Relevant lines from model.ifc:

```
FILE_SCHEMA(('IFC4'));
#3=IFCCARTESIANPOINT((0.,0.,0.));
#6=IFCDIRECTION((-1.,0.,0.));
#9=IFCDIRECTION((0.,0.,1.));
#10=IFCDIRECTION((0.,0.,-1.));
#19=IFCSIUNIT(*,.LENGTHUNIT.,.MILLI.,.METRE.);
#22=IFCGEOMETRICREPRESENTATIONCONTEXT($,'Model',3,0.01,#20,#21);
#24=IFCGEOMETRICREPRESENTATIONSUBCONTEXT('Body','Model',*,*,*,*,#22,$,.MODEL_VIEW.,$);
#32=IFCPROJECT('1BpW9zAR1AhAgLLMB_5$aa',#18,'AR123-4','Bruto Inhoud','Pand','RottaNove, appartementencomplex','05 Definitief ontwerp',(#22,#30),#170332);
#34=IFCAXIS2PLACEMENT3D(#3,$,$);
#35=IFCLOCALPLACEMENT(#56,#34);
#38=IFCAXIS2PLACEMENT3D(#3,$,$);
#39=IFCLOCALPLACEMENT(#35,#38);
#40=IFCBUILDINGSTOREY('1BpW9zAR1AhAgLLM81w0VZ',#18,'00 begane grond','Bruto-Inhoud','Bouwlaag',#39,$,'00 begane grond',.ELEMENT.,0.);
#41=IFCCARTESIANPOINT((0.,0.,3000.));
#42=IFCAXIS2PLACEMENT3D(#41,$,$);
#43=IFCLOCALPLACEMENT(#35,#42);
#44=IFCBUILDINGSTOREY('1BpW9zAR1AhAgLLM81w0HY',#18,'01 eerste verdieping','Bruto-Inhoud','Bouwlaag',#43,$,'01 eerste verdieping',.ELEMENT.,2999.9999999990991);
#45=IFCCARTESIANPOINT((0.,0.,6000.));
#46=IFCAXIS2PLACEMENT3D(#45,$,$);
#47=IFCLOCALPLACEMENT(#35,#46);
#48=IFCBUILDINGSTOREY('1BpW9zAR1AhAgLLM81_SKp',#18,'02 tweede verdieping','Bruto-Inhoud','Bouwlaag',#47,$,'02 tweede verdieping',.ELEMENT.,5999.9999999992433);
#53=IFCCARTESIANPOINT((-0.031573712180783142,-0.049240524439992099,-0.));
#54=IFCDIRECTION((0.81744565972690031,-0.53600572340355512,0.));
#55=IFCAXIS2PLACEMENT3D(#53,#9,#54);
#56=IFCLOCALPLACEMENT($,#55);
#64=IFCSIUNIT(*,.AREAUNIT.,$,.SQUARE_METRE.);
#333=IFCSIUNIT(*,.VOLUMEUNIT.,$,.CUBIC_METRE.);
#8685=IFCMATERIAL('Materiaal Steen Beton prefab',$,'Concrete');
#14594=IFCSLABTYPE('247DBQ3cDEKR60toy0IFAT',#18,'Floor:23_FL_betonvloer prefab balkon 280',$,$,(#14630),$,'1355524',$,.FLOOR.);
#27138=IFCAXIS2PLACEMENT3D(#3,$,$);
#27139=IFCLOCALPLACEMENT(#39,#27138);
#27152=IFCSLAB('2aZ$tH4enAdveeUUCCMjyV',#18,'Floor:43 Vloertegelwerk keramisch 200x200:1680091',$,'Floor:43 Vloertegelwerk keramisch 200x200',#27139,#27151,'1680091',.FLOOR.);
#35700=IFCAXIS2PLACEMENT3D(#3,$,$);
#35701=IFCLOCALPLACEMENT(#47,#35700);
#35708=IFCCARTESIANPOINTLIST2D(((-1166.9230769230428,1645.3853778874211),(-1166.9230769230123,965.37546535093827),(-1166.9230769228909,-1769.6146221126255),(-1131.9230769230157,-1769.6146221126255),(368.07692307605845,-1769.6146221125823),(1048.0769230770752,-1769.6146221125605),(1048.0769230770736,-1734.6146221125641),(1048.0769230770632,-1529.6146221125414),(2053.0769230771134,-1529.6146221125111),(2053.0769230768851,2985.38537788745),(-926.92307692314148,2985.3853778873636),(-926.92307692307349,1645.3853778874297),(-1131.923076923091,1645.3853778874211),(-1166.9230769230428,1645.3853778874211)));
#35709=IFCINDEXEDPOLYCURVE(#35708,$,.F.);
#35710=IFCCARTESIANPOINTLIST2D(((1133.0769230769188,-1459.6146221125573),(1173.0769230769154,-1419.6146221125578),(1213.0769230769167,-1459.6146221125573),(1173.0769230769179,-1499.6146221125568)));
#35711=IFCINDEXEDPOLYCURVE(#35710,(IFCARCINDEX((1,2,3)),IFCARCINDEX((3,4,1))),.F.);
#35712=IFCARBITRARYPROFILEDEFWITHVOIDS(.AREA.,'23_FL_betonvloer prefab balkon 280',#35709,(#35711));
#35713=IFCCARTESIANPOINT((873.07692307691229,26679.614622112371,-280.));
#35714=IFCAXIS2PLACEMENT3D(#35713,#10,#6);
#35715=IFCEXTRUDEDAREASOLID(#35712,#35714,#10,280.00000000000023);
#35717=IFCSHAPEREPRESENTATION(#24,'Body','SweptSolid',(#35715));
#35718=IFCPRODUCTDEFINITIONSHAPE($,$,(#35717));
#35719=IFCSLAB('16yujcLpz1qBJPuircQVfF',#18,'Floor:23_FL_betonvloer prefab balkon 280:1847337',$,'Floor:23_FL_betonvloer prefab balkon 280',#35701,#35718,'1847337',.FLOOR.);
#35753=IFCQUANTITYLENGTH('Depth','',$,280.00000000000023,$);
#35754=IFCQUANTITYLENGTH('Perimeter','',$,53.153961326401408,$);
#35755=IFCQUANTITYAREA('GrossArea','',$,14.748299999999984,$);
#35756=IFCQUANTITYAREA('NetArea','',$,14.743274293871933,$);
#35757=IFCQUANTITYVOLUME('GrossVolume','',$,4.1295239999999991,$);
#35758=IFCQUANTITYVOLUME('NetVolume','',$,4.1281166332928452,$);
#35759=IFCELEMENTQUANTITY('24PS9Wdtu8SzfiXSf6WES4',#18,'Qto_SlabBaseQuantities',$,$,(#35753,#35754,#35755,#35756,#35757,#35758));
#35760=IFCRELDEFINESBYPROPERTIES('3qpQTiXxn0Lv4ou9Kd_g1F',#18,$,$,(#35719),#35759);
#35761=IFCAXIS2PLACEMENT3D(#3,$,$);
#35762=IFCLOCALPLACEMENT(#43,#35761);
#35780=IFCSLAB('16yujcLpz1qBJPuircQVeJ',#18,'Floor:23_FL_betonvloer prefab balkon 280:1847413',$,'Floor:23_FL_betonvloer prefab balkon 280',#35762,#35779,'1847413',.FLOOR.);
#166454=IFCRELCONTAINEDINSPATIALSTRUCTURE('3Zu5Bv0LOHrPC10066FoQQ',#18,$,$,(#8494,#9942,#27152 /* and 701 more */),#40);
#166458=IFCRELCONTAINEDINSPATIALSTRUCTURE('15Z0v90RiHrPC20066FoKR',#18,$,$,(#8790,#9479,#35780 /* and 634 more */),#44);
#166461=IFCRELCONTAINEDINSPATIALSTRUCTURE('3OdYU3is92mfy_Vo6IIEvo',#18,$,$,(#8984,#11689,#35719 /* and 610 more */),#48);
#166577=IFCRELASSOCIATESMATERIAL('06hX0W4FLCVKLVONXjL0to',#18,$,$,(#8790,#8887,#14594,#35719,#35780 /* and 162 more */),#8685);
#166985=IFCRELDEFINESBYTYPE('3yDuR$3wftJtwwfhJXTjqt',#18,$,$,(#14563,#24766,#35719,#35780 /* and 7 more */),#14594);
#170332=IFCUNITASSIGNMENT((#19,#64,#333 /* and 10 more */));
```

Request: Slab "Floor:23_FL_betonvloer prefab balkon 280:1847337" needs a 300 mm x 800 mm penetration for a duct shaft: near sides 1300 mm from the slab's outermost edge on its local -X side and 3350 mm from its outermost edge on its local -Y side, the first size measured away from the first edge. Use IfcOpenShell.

```python
import numpy as np
import ifcopenshell
import ifcopenshell.api.feature
import ifcopenshell.api.geometry
import ifcopenshell.api.pset
import ifcopenshell.api.root
import ifcopenshell.geom
import ifcopenshell.util.element
import ifcopenshell.util.placement
import ifcopenshell.util.representation
import ifcopenshell.util.shape
import ifcopenshell.util.unit

model = ifcopenshell.open("model.ifc")
unit_scale = ifcopenshell.util.unit.calculate_unit_scale(model)
area_scale = ifcopenshell.util.unit.calculate_unit_scale(model, "AREAUNIT")
volume_scale = ifcopenshell.util.unit.calculate_unit_scale(model, "VOLUMEUNIT")
settings = ifcopenshell.geom.settings()


def volume(element):
    """Net volume in cubic metres, openings subtracted."""
    shape = ifcopenshell.geom.create_shape(settings, element)
    return ifcopenshell.util.shape.get_volume(shape.geometry)


slab = model.by_id(35719)
before = volume(slab)

# Extent in the slab's own axes, in metres. The edges named are its -X and -Y sides.
slab_shape = ifcopenshell.geom.create_shape(settings, slab)
vertices = ifcopenshell.util.shape.get_vertices(slab_shape.geometry)
x_min, y_min, bottom = vertices.min(axis=0)
top = vertices[:, 2].max()

opening = ifcopenshell.api.root.create_entity(model, ifc_class="IfcOpeningElement", name="Duct shaft opening", predefined_type="OPENING")
context = ifcopenshell.util.representation.get_context(model, "Model", "Body", "MODEL_VIEW")
width, depth = 0.3, 0.8
outline = [(0.0, 0.0), (width, 0.0), (width, depth), (0.0, depth), (0.0, 0.0)]
# Overshoot both faces by 50 mm so the cut is clean.
shape = ifcopenshell.api.geometry.add_slab_representation(
    model, context=context, depth=top - bottom + 0.1, polyline=outline
)
ifcopenshell.api.geometry.assign_representation(model, product=opening, representation=shape)

matrix = ifcopenshell.util.placement.get_local_placement(slab.ObjectPlacement)
matrix[:, 3] = matrix @ np.append(np.array([x_min + 1.3, y_min + 3.35, bottom - 0.05]) / unit_scale, 1.0)
ifcopenshell.api.geometry.edit_object_placement(model, product=opening, matrix=matrix, is_si=False)
ifcopenshell.api.feature.add_feature(model, feature=opening, element=slab)

after = volume(slab)

# Update the slab's stored quantities.
qto = model.by_id(ifcopenshell.util.element.get_pset(slab, "Qto_SlabBaseQuantities", should_inherit=False)["id"])
ifcopenshell.api.pset.edit_qto(model, qto=qto, properties={
    "NetArea": after / (top - bottom) / area_scale,
    "NetVolume": after / volume_scale,
})

print(f"slab volume {before:.3f} -> {after:.3f} m3")

model.write("model_edited.ifc")
```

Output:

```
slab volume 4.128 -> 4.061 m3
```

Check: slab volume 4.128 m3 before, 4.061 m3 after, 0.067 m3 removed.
